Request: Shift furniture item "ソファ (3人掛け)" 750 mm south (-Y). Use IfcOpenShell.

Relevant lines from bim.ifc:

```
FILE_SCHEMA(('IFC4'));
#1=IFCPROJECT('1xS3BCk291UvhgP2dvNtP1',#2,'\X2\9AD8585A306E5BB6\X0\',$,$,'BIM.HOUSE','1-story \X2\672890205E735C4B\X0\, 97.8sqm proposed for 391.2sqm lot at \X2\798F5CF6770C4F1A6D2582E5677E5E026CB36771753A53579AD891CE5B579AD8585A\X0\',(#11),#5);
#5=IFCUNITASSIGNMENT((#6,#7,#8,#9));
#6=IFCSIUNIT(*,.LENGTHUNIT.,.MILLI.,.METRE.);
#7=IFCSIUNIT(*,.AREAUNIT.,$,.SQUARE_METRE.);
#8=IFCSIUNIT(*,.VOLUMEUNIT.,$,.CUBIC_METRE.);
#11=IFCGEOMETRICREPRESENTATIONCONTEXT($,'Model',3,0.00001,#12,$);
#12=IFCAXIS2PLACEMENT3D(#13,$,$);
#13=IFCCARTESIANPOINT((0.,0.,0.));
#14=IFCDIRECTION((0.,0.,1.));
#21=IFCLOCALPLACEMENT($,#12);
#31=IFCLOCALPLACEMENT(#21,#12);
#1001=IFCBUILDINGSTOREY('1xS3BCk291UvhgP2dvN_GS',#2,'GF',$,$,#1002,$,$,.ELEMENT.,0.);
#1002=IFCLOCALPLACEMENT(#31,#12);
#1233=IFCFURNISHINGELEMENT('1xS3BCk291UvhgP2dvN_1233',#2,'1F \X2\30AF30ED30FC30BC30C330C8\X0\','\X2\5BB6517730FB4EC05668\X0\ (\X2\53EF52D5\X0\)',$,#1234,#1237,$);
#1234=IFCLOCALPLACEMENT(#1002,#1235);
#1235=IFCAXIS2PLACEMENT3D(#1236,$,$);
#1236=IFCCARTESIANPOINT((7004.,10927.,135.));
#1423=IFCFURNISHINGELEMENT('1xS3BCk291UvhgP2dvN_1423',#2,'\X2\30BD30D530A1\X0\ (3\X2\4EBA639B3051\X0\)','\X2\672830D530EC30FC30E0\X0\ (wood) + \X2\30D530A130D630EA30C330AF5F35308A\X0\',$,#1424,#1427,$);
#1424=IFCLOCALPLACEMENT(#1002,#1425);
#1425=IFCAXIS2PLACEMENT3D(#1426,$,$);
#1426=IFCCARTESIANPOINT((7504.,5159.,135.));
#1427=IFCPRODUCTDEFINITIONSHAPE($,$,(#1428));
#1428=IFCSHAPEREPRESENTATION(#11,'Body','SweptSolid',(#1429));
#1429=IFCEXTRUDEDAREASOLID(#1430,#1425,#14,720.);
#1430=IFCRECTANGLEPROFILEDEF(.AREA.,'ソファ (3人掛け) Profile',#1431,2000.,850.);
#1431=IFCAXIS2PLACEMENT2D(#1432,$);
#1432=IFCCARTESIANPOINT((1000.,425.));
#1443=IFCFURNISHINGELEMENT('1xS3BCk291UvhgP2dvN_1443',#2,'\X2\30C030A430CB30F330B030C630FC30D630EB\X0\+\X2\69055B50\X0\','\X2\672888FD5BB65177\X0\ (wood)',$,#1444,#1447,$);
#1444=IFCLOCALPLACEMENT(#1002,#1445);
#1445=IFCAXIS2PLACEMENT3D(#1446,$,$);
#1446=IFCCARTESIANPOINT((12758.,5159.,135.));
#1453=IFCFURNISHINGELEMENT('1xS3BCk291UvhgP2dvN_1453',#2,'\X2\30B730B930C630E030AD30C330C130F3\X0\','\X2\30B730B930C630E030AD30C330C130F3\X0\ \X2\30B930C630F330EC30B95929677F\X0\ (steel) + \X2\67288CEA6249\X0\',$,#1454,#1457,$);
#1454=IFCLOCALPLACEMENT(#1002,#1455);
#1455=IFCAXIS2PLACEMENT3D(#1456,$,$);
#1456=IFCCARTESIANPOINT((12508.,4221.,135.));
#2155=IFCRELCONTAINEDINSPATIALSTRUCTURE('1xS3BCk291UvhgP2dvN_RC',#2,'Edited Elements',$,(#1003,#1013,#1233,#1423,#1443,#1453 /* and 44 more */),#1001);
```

```python
import ifcopenshell
import ifcopenshell.api.geometry
import ifcopenshell.util.placement
import ifcopenshell.util.unit

model = ifcopenshell.open("bim.ifc")
unit_scale = ifcopenshell.util.unit.calculate_unit_scale(model)

item = model.by_id(1423)
matrix = ifcopenshell.util.placement.get_local_placement(item.ObjectPlacement)
matrix[1, 3] -= 0.75 / unit_scale
ifcopenshell.api.geometry.edit_object_placement(model, product=item, matrix=matrix, is_si=False)

print(ifcopenshell.util.placement.get_local_placement(item.ObjectPlacement).round(3) + 0.0)

model.write("bim_updated.ifc")
```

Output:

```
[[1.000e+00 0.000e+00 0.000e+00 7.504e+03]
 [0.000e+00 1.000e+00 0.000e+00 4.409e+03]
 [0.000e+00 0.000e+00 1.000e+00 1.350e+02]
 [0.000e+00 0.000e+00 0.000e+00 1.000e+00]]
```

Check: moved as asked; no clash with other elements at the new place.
